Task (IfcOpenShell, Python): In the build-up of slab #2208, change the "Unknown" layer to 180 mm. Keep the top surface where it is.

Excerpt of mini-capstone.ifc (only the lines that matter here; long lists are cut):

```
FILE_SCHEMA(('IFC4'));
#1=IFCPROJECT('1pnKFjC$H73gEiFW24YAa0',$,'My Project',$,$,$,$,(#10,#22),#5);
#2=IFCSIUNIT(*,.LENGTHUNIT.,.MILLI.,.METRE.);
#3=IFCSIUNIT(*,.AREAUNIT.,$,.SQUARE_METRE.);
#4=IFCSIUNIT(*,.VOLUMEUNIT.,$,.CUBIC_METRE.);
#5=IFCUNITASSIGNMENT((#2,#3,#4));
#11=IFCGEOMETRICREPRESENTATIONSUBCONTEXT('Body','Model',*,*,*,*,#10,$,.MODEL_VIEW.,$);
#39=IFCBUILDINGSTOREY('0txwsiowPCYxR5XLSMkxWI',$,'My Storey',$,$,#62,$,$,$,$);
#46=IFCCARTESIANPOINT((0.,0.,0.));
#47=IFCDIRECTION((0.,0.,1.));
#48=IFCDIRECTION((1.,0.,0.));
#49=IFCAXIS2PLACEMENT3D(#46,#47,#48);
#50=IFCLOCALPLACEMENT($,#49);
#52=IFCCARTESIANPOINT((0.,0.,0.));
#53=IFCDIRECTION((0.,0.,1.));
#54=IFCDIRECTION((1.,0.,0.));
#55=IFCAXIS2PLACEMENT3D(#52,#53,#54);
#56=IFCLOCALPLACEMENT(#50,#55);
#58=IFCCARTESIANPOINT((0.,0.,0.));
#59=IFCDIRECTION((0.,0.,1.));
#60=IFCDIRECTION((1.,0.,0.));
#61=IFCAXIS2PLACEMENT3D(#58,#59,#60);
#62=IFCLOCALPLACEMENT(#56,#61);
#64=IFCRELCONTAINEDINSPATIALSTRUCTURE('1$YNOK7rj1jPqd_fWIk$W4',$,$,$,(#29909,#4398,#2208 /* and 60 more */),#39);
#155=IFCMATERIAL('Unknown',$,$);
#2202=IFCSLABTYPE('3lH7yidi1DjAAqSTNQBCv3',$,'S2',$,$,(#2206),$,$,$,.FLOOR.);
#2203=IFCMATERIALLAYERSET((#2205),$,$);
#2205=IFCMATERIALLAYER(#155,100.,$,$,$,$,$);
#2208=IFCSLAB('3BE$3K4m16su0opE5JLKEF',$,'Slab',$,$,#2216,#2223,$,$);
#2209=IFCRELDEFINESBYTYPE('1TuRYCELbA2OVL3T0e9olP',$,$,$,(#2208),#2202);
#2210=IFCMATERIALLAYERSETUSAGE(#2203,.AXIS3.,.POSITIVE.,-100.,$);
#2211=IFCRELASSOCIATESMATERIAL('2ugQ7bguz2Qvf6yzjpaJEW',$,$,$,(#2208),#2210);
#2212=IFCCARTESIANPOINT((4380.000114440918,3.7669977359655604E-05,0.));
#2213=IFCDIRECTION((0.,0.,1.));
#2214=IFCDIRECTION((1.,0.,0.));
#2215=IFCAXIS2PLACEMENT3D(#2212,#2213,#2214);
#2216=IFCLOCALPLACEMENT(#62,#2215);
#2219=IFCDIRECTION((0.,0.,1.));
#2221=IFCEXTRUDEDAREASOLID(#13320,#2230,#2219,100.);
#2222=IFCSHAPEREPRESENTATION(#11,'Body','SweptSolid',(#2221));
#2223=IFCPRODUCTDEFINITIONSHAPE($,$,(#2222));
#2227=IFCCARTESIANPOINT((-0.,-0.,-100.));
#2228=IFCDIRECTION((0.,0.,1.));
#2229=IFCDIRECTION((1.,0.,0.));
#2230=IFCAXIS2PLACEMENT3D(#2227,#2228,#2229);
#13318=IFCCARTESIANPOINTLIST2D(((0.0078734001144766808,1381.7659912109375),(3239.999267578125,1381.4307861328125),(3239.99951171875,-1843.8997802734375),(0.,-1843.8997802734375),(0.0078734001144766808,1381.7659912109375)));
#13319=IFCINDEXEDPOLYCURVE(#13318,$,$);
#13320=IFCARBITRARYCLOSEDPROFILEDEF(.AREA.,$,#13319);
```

```python
import ifcopenshell
import ifcopenshell.util.element
import ifcopenshell.util.representation
import ifcopenshell.util.unit

model = ifcopenshell.open("mini-capstone.ifc")
unit_scale = ifcopenshell.util.unit.calculate_unit_scale(model)

layer_set = model.by_id(2203)
layer = next(l for l in layer_set.MaterialLayers if l.Material and l.Material.Name == "Unknown")
change = 0.18 / unit_scale - layer.LayerThickness
layer.LayerThickness += change

# Geometry does not follow the layer set by itself.
slabs = [e for e in ifcopenshell.util.element.get_elements_by_material(model, layer_set) if e.is_a("IfcSlab")]
for slab in sorted(slabs, key=lambda e: e.id()):
    body = ifcopenshell.util.representation.get_representation(slab, "Model", "Body")
    solid = body.Items[0]
    old_depth = solid.Depth
    solid.Depth += change
    # Extruded upwards: lower the start of the extrusion so the top stays.
    x, y, z = solid.Position.Location.Coordinates
    solid.Position.Location = model.createIfcCartesianPoint((x, y, z - change))
    print(slab.id(), f"{old_depth:g} -> {solid.Depth:g}")

# The layers are counted up from the underside, which has moved.
for usage in {ifcopenshell.util.element.get_material(slab) for slab in slabs}:
    usage.OffsetFromReferenceLine -= change

model.write("mini-capstone-out.ifc")
```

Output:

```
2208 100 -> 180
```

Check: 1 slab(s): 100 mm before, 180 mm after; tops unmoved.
